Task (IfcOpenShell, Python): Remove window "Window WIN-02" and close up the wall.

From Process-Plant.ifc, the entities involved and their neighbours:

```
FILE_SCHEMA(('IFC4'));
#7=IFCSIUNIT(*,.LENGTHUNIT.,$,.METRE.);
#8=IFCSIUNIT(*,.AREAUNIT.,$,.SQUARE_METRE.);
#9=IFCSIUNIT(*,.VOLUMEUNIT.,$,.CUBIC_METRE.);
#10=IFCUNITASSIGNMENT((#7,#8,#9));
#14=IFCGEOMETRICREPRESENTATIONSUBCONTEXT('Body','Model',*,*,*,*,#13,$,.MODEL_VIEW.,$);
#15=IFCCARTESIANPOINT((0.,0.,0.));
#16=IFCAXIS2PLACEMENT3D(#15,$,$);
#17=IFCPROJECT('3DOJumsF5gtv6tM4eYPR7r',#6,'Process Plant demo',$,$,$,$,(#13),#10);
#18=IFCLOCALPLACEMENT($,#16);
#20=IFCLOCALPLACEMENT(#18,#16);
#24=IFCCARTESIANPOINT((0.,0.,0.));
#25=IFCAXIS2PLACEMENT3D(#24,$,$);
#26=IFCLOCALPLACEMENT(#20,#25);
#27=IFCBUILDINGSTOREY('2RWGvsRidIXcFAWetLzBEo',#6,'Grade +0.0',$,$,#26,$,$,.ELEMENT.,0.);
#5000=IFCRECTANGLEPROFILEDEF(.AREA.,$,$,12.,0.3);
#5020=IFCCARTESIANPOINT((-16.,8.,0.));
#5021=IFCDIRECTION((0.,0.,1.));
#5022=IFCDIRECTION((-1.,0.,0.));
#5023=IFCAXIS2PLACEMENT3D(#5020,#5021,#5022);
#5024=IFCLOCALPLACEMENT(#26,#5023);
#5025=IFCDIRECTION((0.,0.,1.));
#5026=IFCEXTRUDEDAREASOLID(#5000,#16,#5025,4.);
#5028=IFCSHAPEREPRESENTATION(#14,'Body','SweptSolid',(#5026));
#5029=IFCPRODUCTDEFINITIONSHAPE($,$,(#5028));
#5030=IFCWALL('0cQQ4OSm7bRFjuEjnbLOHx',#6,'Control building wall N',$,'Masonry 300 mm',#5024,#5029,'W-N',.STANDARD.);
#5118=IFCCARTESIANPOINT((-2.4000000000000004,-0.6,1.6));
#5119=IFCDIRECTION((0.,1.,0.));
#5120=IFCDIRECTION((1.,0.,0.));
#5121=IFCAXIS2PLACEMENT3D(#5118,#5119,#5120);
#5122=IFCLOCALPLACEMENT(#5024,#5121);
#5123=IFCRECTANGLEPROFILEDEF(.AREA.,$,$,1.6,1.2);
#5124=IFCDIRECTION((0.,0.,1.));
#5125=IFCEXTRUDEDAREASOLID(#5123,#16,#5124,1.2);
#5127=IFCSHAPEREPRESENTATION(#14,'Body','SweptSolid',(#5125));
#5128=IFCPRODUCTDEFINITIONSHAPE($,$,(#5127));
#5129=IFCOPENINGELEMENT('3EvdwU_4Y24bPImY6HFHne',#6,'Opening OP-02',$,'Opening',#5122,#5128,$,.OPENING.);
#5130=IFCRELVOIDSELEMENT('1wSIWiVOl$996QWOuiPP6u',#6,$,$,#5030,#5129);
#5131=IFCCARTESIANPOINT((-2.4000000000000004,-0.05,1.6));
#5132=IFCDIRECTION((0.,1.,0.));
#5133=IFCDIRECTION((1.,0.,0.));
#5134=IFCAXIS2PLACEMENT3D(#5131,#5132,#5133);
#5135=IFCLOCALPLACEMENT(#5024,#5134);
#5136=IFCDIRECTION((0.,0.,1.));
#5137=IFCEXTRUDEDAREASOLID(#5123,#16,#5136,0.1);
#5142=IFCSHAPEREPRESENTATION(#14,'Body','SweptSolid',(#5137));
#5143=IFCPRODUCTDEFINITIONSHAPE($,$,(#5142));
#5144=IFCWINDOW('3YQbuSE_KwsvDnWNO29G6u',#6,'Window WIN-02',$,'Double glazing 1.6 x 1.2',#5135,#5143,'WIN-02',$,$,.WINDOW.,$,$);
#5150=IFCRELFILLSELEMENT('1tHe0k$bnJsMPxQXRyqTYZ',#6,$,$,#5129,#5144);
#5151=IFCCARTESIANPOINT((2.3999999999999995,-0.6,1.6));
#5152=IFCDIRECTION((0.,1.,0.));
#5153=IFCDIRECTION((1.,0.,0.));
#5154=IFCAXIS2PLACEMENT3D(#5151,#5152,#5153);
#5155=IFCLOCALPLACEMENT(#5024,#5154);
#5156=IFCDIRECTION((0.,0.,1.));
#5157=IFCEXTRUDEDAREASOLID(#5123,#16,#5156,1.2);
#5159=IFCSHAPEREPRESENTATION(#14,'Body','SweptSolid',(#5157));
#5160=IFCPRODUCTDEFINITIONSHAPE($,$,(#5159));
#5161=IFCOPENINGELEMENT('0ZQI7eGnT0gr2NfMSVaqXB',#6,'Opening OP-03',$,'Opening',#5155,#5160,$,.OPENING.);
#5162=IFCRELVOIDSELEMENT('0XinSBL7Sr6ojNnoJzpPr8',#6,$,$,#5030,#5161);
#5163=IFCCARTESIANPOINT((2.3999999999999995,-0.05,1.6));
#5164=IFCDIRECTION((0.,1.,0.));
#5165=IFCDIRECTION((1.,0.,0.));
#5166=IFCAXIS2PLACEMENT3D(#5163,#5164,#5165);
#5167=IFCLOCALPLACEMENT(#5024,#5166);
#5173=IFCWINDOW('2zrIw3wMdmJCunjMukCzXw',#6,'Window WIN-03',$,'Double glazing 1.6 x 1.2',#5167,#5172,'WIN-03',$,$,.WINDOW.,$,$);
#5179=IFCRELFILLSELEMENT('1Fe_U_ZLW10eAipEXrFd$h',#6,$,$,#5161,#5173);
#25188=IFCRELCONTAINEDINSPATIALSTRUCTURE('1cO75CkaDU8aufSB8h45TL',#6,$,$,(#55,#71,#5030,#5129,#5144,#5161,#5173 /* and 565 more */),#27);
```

```python
import ifcopenshell
import ifcopenshell.api.feature
import ifcopenshell.api.root
import ifcopenshell.geom
import ifcopenshell.util.shape

model = ifcopenshell.open("Process-Plant.ifc")
settings = ifcopenshell.geom.settings()


def volume(element):
    """Net volume in cubic metres, openings subtracted."""
    shape = ifcopenshell.geom.create_shape(settings, element)
    return ifcopenshell.util.shape.get_volume(shape.geometry)


window = model.by_guid("3YQbuSE_KwsvDnWNO29G6u")
opening = window.FillsVoids[0].RelatingOpeningElement
wall = opening.VoidsElements[0].RelatingBuildingElement
before = volume(wall)

ifcopenshell.api.root.remove_product(model, product=window)
ifcopenshell.api.feature.remove_feature(model, feature=opening)

after = volume(wall)

print(f"wall volume {before:.3f} -> {after:.3f} m3")

model.write("Process-Plant_edited.ifc")
```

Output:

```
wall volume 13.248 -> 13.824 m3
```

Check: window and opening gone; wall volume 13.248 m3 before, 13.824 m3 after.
